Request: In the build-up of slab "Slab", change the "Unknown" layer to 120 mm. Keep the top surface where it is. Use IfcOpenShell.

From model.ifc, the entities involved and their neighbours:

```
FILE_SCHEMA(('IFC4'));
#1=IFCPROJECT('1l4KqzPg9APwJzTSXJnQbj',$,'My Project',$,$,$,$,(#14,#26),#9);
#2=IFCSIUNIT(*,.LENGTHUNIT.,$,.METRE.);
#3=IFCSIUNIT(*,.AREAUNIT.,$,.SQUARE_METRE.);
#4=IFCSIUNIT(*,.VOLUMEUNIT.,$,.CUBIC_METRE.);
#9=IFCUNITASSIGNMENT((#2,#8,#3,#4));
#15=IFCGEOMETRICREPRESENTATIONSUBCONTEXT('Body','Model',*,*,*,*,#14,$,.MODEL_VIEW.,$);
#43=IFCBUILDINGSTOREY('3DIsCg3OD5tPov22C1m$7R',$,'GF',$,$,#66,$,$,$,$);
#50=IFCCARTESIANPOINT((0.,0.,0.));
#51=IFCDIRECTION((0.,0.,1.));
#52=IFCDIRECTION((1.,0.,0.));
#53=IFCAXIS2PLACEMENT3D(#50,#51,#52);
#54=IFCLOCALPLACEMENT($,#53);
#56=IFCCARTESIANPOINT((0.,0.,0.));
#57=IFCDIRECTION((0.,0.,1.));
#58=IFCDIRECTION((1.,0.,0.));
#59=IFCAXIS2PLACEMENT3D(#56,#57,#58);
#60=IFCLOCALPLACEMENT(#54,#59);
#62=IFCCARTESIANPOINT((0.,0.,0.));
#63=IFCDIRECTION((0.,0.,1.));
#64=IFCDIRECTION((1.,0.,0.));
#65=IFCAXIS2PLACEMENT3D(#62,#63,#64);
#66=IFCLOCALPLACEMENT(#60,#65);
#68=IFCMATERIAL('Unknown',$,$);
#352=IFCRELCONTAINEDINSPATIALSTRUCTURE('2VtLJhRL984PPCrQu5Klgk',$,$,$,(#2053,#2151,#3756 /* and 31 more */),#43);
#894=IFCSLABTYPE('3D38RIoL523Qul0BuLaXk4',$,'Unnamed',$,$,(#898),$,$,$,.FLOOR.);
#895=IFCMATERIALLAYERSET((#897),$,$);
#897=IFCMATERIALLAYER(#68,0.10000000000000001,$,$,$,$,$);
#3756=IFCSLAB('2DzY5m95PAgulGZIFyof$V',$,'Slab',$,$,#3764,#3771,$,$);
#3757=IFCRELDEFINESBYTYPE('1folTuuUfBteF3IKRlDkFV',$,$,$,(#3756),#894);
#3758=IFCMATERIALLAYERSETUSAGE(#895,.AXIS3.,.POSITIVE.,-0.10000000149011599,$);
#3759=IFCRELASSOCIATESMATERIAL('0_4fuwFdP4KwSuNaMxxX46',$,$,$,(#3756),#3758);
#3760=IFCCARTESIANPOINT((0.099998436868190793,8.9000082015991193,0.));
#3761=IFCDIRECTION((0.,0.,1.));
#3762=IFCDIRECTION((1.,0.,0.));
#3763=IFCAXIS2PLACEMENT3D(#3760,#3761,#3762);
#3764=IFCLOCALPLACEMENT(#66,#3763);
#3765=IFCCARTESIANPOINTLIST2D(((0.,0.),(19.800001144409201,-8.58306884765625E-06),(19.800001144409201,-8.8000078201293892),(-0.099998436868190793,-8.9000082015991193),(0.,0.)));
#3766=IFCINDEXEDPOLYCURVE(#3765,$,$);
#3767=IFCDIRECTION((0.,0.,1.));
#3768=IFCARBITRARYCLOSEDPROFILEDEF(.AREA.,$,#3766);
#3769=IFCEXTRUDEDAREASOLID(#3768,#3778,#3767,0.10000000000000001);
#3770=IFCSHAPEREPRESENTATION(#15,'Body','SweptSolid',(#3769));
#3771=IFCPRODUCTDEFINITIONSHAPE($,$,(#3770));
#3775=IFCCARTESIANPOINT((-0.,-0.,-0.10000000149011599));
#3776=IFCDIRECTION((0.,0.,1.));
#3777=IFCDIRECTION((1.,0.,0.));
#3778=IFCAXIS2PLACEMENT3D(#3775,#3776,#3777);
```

```python
import ifcopenshell
import ifcopenshell.util.element
import ifcopenshell.util.representation
import ifcopenshell.util.unit

model = ifcopenshell.open("model.ifc")
unit_scale = ifcopenshell.util.unit.calculate_unit_scale(model)

layer_set = model.by_id(895)
layer = next(l for l in layer_set.MaterialLayers if l.Material and l.Material.Name == "Unknown")
change = 0.12 / unit_scale - layer.LayerThickness
layer.LayerThickness += change

# Geometry does not follow the layer set by itself.
slabs = [e for e in ifcopenshell.util.element.get_elements_by_material(model, layer_set) if e.is_a("IfcSlab")]
for slab in sorted(slabs, key=lambda e: e.id()):
    body = ifcopenshell.util.representation.get_representation(slab, "Model", "Body")
    solid = body.Items[0]
    old_depth = solid.Depth
    solid.Depth += change
    # Extruded upwards: lower the start of the extrusion so the top stays.
    x, y, z = solid.Position.Location.Coordinates
    solid.Position.Location = model.createIfcCartesianPoint((x, y, z - change))
    print(slab.id(), f"{old_depth:g} -> {solid.Depth:g}")

# The layers are counted up from the underside, which has moved.
for usage in {ifcopenshell.util.element.get_material(slab) for slab in slabs}:
    usage.OffsetFromReferenceLine -= change

model.write("model_updated.ifc")
```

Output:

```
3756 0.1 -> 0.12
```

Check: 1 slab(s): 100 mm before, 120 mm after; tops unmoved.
